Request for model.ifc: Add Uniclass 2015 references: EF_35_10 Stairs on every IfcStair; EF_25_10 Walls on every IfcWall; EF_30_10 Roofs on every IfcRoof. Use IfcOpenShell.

First a look at what the model holds.

```python
import ifcopenshell

model = ifcopenshell.open("model.ifc")
print(model.schema)
print("classifications:", [c.Name for c in model.by_type("IfcClassification")])
for ifc_class in ("IfcDoor", "IfcRoof", "IfcStair", "IfcWall", "IfcWindow"):
    print(ifc_class, len(model.by_type(ifc_class)))
```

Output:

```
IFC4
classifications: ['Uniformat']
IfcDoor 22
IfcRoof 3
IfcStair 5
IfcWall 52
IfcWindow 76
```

```python
import ifcopenshell
import ifcopenshell.api.classification

model = ifcopenshell.open("model.ifc")

system = ifcopenshell.api.classification.add_classification(model, classification="Uniclass 2015")

codes = {
    "IfcStair": ("EF_35_10", "Stairs"),
    "IfcWall": ("EF_25_10", "Walls"),
    "IfcRoof": ("EF_30_10", "Roofs"),
}
for ifc_class, (code, name) in codes.items():
    products = model.by_type(ifc_class)
    ifcopenshell.api.classification.add_reference(
        model, products=products, classification=system, identification=code, name=name
    )
    print(code, len(products))

model.write("model_updated.ifc")
```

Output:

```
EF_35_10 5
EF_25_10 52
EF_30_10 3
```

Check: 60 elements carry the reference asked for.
